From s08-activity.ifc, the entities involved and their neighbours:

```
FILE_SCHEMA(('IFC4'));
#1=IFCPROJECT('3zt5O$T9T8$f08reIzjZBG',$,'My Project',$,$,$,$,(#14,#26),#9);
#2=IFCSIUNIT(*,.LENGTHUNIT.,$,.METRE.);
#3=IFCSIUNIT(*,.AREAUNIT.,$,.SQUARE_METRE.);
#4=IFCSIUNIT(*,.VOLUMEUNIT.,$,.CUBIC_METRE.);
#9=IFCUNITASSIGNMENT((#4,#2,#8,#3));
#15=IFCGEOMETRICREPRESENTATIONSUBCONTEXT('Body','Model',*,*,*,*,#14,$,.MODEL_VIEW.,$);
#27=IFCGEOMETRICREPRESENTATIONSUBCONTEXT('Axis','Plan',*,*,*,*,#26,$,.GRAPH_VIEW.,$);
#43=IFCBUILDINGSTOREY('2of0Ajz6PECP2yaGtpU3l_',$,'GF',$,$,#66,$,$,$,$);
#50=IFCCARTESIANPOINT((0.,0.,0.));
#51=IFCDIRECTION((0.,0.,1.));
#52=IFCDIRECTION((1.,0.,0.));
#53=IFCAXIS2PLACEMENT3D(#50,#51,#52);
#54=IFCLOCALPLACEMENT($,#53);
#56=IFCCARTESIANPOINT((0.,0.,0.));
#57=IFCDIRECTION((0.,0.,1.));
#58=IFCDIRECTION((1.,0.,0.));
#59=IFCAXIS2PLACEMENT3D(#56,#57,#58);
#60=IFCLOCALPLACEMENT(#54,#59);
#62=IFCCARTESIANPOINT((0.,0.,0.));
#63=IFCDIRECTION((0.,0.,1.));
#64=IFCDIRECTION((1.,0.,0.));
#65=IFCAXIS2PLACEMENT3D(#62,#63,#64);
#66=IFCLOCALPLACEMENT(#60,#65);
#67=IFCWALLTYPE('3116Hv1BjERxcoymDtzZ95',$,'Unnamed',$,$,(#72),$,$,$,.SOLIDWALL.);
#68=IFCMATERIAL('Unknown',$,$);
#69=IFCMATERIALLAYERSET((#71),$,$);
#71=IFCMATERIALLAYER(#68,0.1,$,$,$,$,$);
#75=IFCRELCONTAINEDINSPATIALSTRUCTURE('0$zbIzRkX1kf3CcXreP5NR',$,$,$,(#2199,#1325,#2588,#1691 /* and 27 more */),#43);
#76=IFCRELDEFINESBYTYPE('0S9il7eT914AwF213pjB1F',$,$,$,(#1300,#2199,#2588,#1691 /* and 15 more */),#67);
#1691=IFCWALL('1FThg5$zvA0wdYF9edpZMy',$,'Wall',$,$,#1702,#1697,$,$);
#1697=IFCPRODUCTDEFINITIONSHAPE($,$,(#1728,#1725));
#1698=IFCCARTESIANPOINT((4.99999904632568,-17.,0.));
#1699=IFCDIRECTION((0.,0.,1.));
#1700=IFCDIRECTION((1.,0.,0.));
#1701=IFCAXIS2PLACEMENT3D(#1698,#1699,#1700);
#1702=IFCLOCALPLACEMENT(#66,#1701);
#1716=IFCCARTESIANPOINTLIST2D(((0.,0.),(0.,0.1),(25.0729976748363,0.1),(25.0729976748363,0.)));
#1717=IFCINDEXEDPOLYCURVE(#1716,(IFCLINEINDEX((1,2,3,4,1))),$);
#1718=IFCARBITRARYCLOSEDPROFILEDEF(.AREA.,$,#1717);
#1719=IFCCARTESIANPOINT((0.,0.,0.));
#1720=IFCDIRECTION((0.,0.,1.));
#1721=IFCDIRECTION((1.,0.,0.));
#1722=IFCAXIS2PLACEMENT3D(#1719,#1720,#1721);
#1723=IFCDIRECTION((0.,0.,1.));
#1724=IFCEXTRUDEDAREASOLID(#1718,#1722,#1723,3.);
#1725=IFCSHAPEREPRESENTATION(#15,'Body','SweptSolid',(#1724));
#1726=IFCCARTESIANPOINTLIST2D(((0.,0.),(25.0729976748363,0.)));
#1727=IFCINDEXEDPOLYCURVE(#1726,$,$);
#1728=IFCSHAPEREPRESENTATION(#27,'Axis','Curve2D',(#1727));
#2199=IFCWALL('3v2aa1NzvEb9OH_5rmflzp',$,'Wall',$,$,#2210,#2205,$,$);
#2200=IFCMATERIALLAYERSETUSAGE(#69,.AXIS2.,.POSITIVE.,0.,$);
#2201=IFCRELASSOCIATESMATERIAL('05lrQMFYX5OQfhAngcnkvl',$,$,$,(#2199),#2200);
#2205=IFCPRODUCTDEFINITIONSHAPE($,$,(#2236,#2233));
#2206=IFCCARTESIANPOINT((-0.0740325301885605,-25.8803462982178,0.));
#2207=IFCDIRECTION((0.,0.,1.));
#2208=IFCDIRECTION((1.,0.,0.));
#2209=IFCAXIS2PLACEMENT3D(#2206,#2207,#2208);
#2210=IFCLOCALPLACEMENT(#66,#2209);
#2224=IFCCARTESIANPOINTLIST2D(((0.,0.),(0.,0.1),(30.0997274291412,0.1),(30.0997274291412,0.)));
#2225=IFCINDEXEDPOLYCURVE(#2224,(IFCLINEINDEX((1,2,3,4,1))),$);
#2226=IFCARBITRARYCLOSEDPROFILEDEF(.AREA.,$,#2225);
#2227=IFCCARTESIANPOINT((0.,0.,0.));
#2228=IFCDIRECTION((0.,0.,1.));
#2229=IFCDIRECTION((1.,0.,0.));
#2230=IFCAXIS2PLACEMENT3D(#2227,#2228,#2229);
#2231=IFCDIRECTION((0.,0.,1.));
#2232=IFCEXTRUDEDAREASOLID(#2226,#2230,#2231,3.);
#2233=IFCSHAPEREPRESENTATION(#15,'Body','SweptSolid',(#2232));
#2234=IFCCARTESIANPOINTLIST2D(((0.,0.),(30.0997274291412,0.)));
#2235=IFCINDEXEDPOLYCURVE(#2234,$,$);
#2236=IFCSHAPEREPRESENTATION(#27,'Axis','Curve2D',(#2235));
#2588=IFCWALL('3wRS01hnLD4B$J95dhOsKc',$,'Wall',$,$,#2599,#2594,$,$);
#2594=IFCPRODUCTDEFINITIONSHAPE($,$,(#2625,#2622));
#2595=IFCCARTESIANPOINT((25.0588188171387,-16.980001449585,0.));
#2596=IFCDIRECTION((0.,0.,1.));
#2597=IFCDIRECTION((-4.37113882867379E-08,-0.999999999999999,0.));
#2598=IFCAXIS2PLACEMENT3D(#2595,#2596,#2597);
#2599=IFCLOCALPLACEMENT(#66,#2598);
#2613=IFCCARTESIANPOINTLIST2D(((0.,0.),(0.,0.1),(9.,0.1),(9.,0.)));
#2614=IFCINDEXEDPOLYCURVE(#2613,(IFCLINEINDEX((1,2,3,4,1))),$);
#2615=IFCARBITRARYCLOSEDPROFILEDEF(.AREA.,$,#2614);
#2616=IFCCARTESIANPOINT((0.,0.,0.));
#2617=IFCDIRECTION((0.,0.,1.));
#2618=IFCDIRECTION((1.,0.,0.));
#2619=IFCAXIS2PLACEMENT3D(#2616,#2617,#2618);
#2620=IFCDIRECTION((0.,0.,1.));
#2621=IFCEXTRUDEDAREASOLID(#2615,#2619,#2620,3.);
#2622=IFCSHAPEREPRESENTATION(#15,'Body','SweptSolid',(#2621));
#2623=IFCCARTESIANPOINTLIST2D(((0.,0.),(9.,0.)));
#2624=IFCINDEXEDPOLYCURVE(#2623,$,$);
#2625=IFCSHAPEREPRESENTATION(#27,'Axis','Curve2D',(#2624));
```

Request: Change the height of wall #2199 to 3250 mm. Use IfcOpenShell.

```python
import ifcopenshell
import ifcopenshell.geom
import ifcopenshell.util.representation
import ifcopenshell.util.shape

model = ifcopenshell.open("s08-activity.ifc")
settings = ifcopenshell.geom.settings()


def volume(element):
    """Net volume in cubic metres, openings subtracted."""
    shape = ifcopenshell.geom.create_shape(settings, element)
    return ifcopenshell.util.shape.get_volume(shape.geometry)


wall = model.by_id(2199)
before = volume(wall)

body = ifcopenshell.util.representation.get_representation(wall, "Model", "Body")
solid = body.Items[0]
old_height = solid.Depth
solid.Depth = 3.25
after = volume(wall)

print(f"height {old_height:g} -> {solid.Depth:g}, volume {before:.3f} -> {after:.3f} m3")

model.write("s08-activity_updated.ifc")
```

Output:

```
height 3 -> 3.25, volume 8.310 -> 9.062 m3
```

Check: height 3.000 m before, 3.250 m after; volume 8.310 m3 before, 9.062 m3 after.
